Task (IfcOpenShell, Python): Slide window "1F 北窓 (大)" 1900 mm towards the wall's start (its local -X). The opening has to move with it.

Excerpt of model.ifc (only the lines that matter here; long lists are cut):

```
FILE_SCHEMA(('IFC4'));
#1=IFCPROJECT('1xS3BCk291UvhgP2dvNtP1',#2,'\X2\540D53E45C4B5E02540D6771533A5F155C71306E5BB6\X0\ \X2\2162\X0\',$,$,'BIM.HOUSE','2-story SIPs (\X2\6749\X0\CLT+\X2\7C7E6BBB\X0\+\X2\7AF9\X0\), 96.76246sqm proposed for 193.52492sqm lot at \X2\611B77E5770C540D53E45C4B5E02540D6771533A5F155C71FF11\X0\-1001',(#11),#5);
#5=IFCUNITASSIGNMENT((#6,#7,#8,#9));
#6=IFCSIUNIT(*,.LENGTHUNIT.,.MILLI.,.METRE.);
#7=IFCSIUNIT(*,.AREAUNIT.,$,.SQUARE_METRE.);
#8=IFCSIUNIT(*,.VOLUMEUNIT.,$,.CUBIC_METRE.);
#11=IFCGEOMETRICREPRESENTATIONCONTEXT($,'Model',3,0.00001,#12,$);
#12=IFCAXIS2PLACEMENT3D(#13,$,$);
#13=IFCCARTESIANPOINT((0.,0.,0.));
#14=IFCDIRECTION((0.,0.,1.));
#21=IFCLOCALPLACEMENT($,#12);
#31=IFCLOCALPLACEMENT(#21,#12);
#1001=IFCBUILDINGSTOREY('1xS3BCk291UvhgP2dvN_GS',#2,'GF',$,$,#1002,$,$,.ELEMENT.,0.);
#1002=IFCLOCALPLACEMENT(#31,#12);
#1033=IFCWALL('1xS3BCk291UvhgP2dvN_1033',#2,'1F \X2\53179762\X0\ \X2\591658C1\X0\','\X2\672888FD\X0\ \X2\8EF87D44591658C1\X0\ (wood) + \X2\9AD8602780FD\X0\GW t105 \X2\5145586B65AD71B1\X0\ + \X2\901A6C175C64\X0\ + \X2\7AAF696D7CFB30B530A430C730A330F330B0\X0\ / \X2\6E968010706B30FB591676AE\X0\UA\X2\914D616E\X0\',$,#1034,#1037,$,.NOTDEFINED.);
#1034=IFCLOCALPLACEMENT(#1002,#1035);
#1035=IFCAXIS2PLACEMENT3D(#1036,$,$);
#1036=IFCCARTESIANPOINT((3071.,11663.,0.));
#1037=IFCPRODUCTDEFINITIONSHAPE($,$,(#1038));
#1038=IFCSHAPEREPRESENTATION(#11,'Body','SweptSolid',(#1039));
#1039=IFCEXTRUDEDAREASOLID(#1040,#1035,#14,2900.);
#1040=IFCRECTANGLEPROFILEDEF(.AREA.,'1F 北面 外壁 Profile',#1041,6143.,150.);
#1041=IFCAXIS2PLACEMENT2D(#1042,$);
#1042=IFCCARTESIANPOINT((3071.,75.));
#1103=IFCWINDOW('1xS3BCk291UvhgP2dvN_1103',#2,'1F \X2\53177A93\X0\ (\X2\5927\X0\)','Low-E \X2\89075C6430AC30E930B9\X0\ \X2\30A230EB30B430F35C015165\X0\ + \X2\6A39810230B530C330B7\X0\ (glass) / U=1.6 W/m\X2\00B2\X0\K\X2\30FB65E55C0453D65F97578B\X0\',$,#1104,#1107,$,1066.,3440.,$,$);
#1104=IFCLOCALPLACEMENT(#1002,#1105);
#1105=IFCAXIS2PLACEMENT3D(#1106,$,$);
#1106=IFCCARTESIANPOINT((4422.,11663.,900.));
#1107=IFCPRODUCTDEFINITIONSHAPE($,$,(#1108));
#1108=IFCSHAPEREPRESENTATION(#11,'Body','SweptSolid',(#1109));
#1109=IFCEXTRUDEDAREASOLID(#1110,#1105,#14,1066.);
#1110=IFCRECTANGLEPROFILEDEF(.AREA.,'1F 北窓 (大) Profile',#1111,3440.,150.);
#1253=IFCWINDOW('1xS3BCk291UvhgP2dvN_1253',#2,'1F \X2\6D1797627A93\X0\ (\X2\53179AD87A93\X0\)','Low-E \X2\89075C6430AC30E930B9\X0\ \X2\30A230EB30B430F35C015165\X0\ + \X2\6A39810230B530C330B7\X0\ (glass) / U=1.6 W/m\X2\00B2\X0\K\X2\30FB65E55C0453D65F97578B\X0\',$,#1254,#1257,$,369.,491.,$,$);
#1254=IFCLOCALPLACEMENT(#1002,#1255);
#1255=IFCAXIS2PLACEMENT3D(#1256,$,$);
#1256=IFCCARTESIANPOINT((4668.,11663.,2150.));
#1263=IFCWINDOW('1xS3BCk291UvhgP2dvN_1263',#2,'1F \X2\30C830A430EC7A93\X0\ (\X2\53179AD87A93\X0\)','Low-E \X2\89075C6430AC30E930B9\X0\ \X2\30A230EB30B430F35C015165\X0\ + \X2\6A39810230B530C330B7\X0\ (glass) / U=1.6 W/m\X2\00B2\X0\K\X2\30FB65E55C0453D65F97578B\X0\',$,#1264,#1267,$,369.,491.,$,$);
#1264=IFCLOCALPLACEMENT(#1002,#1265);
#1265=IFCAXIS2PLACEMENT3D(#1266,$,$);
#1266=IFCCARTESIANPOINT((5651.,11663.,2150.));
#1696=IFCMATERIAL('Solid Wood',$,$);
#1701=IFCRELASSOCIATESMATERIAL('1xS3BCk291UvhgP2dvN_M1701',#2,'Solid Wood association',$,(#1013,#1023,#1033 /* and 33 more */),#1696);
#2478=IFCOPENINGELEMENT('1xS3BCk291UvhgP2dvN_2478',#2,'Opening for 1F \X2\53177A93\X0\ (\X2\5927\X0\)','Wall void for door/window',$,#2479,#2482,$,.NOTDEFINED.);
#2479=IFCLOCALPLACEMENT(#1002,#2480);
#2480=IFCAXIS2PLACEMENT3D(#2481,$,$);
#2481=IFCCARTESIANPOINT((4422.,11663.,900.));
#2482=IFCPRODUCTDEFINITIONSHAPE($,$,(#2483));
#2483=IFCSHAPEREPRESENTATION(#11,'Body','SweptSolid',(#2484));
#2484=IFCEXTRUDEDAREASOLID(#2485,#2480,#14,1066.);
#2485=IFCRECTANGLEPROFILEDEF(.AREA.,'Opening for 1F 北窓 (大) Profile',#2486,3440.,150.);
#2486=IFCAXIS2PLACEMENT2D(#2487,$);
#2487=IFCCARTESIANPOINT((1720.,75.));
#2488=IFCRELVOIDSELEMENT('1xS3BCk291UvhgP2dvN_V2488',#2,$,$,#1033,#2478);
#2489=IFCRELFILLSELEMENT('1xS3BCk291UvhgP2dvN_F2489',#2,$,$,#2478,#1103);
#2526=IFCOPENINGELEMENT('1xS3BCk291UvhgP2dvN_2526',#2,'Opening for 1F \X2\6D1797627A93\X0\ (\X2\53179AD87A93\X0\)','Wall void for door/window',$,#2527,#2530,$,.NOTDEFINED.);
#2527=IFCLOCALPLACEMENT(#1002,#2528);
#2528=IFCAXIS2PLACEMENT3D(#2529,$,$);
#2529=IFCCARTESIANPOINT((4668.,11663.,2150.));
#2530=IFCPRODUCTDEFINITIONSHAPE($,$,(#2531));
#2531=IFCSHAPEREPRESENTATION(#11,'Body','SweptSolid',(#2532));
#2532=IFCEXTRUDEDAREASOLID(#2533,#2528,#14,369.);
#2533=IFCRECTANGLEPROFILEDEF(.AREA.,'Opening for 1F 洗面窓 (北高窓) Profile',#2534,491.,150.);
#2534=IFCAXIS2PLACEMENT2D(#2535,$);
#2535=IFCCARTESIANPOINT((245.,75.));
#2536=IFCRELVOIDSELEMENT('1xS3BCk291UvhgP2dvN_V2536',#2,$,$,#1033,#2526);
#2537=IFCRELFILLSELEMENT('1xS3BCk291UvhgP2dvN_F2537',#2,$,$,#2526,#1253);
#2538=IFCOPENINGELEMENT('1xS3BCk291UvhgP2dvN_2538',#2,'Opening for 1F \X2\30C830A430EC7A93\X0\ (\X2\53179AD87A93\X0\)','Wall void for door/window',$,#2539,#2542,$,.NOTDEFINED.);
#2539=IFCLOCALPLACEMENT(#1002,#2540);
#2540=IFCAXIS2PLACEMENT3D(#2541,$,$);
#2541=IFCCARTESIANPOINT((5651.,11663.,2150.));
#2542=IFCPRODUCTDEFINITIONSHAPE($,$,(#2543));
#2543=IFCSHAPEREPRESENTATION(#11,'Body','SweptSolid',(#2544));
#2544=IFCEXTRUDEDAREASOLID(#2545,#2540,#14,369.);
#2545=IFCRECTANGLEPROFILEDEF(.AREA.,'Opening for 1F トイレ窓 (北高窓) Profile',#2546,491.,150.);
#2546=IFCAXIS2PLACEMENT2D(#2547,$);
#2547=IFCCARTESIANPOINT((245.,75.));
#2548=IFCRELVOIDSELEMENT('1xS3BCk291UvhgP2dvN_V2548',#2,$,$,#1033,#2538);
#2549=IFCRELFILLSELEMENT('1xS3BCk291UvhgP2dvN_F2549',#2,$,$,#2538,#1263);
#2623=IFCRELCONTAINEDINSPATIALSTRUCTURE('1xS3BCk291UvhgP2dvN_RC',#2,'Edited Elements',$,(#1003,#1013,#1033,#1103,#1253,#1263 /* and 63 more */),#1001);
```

```python
import ifcopenshell
import ifcopenshell.api.geometry
import ifcopenshell.util.placement

model = ifcopenshell.open("model.ifc")

window = model.by_guid("1xS3BCk291UvhgP2dvN_1103")
opening = window.FillsVoids[0].RelatingOpeningElement
wall = opening.VoidsElements[0].RelatingBuildingElement

wall_matrix = ifcopenshell.util.placement.get_local_placement(wall.ObjectPlacement)
shift = wall_matrix[:3, 0] * -1900.0
before = ifcopenshell.util.placement.get_local_placement(window.ObjectPlacement)[:3, 3].copy()

# The window is not placed relative to its opening, so move both.
for product in (opening, window):
    matrix = ifcopenshell.util.placement.get_local_placement(product.ObjectPlacement)
    matrix[:3, 3] += shift
    ifcopenshell.api.geometry.edit_object_placement(model, product=product, matrix=matrix, is_si=False)

after = ifcopenshell.util.placement.get_local_placement(window.ObjectPlacement)[:3, 3]
print("window moved by", (after - before).round(3) + 0.0)

model.write("model-out.ifc")
```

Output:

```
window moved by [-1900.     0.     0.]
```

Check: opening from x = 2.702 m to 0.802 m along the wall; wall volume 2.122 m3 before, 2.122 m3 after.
